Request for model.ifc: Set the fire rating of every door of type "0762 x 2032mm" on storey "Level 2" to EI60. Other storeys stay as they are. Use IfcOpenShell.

First a look at what the model holds.

```python
import ifcopenshell
import ifcopenshell.util.element

model = ifcopenshell.open("model.ifc")
print(model.schema)
storey = next(s for s in model.by_type("IfcBuildingStorey") if s.Name == "Level 2")
doors = [e for e in ifcopenshell.util.element.get_decomposition(storey) if e.is_a("IfcDoor")]
seen = {}
for e in doors:
    element_type = ifcopenshell.util.element.get_type(e)
    key = (element_type.Name if element_type != e and element_type else None, ifcopenshell.util.element.get_pset(e, "Pset_DoorCommon", "FireRating"))
    seen[key] = seen.get(key, 0) + 1
for (name, value), count in sorted(seen.items(), key=str):
    print(count, "x", name, "|", value)
```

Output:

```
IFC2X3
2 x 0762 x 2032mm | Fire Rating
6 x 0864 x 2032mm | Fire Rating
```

```python
import ifcopenshell
import ifcopenshell.api.pset
import ifcopenshell.util.element

model = ifcopenshell.open("model.ifc")

storey = next(s for s in model.by_type("IfcBuildingStorey") if s.Name == "Level 2")
doors = [e for e in ifcopenshell.util.element.get_decomposition(storey) if e.is_a("IfcDoor")]

count = 0
for e in doors:
    element_type = ifcopenshell.util.element.get_type(e)
    if element_type in (None, e) or element_type.Name != "0762 x 2032mm":
        continue
    # add_pset returns the element's existing set when there is one.
    pset = ifcopenshell.api.pset.add_pset(model, product=e, name="Pset_DoorCommon")
    ifcopenshell.api.pset.edit_pset(model, pset=pset, properties={"FireRating": "EI60"})
    count += 1

print(count, "doors updated")

model.write("model-out.ifc")
```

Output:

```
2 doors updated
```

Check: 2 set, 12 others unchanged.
